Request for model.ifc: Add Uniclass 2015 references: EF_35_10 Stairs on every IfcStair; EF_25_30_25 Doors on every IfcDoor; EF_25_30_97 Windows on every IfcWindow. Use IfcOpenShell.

First a look at what the model holds.

```python
import ifcopenshell

model = ifcopenshell.open("model.ifc")
print(model.schema)
print("classifications:", [c.Name for c in model.by_type("IfcClassification")])
for ifc_class in ("IfcDoor", "IfcRoof", "IfcStair", "IfcWall", "IfcWindow"):
    print(ifc_class, len(model.by_type(ifc_class)))
```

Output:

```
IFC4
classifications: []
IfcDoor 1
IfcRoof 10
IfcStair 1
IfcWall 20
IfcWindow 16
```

```python
import ifcopenshell
import ifcopenshell.api.classification

model = ifcopenshell.open("model.ifc")

system = ifcopenshell.api.classification.add_classification(model, classification="Uniclass 2015")

codes = {
    "IfcStair": ("EF_35_10", "Stairs"),
    "IfcDoor": ("EF_25_30_25", "Doors"),
    "IfcWindow": ("EF_25_30_97", "Windows"),
}
for ifc_class, (code, name) in codes.items():
    products = model.by_type(ifc_class)
    ifcopenshell.api.classification.add_reference(
        model, products=products, classification=system, identification=code, name=name
    )
    print(code, len(products))

model.write("model_v2.ifc")
```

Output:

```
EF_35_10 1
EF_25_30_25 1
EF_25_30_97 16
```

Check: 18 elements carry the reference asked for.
